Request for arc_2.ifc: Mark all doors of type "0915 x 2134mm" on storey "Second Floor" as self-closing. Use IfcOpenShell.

First a look at what the model holds.

```python
import ifcopenshell
import ifcopenshell.util.element

model = ifcopenshell.open("arc_2.ifc")
print(model.schema)
storey = next(s for s in model.by_type("IfcBuildingStorey") if s.Name == "Second Floor")
doors = [e for e in ifcopenshell.util.element.get_decomposition(storey) if e.is_a("IfcDoor")]
seen = {}
for e in doors:
    element_type = ifcopenshell.util.element.get_type(e)
    key = (element_type.Name if element_type != e and element_type else None, ifcopenshell.util.element.get_pset(e, "Pset_DoorCommon", "SelfClosing"))
    seen[key] = seen.get(key, 0) + 1
for (name, value), count in sorted(seen.items(), key=str):
    print(count, "x", name, "|", value)
```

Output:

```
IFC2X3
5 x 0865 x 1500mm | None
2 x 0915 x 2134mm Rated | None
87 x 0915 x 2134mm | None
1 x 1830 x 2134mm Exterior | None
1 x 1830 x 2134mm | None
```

```python
import ifcopenshell
import ifcopenshell.api.pset
import ifcopenshell.util.element

model = ifcopenshell.open("arc_2.ifc")

storey = next(s for s in model.by_type("IfcBuildingStorey") if s.Name == "Second Floor")
doors = [e for e in ifcopenshell.util.element.get_decomposition(storey) if e.is_a("IfcDoor")]

count = 0
for e in doors:
    element_type = ifcopenshell.util.element.get_type(e)
    if element_type in (None, e) or element_type.Name != "0915 x 2134mm":
        continue
    # add_pset returns the element's existing set when there is one.
    pset = ifcopenshell.api.pset.add_pset(model, product=e, name="Pset_DoorCommon")
    ifcopenshell.api.pset.edit_pset(model, pset=pset, properties={"SelfClosing": True})
    count += 1

print(count, "doors updated")

model.write("arc_2_rev.ifc")
```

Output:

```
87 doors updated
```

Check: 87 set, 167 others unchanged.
